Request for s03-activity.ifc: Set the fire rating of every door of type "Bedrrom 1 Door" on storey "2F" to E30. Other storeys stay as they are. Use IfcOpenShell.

First a look at what the model holds.

```python
import ifcopenshell
import ifcopenshell.util.element

model = ifcopenshell.open("s03-activity.ifc")
print(model.schema)
storey = next(s for s in model.by_type("IfcBuildingStorey") if s.Name == "2F")
doors = [e for e in ifcopenshell.util.element.get_decomposition(storey) if e.is_a("IfcDoor")]
seen = {}
for e in doors:
    element_type = ifcopenshell.util.element.get_type(e)
    key = (element_type.Name if element_type != e and element_type else None, ifcopenshell.util.element.get_pset(e, "Pset_DoorCommon", "FireRating"))
    seen[key] = seen.get(key, 0) + 1
for (name, value), count in sorted(seen.items(), key=str):
    print(count, "x", name, "|", value)
```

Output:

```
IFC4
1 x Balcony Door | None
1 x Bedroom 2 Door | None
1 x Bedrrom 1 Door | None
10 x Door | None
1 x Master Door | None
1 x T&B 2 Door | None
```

```python
import ifcopenshell
import ifcopenshell.api.pset
import ifcopenshell.util.element

model = ifcopenshell.open("s03-activity.ifc")

storey = next(s for s in model.by_type("IfcBuildingStorey") if s.Name == "2F")
doors = [e for e in ifcopenshell.util.element.get_decomposition(storey) if e.is_a("IfcDoor")]

count = 0
for e in doors:
    element_type = ifcopenshell.util.element.get_type(e)
    if element_type in (None, e) or element_type.Name != "Bedrrom 1 Door":
        continue
    # add_pset returns the element's existing set when there is one.
    pset = ifcopenshell.api.pset.add_pset(model, product=e, name="Pset_DoorCommon")
    ifcopenshell.api.pset.edit_pset(model, pset=pset, properties={"FireRating": "E30"})
    count += 1

print(count, "doors updated")

model.write("s03-activity_rev.ifc")
```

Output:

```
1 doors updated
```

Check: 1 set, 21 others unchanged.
